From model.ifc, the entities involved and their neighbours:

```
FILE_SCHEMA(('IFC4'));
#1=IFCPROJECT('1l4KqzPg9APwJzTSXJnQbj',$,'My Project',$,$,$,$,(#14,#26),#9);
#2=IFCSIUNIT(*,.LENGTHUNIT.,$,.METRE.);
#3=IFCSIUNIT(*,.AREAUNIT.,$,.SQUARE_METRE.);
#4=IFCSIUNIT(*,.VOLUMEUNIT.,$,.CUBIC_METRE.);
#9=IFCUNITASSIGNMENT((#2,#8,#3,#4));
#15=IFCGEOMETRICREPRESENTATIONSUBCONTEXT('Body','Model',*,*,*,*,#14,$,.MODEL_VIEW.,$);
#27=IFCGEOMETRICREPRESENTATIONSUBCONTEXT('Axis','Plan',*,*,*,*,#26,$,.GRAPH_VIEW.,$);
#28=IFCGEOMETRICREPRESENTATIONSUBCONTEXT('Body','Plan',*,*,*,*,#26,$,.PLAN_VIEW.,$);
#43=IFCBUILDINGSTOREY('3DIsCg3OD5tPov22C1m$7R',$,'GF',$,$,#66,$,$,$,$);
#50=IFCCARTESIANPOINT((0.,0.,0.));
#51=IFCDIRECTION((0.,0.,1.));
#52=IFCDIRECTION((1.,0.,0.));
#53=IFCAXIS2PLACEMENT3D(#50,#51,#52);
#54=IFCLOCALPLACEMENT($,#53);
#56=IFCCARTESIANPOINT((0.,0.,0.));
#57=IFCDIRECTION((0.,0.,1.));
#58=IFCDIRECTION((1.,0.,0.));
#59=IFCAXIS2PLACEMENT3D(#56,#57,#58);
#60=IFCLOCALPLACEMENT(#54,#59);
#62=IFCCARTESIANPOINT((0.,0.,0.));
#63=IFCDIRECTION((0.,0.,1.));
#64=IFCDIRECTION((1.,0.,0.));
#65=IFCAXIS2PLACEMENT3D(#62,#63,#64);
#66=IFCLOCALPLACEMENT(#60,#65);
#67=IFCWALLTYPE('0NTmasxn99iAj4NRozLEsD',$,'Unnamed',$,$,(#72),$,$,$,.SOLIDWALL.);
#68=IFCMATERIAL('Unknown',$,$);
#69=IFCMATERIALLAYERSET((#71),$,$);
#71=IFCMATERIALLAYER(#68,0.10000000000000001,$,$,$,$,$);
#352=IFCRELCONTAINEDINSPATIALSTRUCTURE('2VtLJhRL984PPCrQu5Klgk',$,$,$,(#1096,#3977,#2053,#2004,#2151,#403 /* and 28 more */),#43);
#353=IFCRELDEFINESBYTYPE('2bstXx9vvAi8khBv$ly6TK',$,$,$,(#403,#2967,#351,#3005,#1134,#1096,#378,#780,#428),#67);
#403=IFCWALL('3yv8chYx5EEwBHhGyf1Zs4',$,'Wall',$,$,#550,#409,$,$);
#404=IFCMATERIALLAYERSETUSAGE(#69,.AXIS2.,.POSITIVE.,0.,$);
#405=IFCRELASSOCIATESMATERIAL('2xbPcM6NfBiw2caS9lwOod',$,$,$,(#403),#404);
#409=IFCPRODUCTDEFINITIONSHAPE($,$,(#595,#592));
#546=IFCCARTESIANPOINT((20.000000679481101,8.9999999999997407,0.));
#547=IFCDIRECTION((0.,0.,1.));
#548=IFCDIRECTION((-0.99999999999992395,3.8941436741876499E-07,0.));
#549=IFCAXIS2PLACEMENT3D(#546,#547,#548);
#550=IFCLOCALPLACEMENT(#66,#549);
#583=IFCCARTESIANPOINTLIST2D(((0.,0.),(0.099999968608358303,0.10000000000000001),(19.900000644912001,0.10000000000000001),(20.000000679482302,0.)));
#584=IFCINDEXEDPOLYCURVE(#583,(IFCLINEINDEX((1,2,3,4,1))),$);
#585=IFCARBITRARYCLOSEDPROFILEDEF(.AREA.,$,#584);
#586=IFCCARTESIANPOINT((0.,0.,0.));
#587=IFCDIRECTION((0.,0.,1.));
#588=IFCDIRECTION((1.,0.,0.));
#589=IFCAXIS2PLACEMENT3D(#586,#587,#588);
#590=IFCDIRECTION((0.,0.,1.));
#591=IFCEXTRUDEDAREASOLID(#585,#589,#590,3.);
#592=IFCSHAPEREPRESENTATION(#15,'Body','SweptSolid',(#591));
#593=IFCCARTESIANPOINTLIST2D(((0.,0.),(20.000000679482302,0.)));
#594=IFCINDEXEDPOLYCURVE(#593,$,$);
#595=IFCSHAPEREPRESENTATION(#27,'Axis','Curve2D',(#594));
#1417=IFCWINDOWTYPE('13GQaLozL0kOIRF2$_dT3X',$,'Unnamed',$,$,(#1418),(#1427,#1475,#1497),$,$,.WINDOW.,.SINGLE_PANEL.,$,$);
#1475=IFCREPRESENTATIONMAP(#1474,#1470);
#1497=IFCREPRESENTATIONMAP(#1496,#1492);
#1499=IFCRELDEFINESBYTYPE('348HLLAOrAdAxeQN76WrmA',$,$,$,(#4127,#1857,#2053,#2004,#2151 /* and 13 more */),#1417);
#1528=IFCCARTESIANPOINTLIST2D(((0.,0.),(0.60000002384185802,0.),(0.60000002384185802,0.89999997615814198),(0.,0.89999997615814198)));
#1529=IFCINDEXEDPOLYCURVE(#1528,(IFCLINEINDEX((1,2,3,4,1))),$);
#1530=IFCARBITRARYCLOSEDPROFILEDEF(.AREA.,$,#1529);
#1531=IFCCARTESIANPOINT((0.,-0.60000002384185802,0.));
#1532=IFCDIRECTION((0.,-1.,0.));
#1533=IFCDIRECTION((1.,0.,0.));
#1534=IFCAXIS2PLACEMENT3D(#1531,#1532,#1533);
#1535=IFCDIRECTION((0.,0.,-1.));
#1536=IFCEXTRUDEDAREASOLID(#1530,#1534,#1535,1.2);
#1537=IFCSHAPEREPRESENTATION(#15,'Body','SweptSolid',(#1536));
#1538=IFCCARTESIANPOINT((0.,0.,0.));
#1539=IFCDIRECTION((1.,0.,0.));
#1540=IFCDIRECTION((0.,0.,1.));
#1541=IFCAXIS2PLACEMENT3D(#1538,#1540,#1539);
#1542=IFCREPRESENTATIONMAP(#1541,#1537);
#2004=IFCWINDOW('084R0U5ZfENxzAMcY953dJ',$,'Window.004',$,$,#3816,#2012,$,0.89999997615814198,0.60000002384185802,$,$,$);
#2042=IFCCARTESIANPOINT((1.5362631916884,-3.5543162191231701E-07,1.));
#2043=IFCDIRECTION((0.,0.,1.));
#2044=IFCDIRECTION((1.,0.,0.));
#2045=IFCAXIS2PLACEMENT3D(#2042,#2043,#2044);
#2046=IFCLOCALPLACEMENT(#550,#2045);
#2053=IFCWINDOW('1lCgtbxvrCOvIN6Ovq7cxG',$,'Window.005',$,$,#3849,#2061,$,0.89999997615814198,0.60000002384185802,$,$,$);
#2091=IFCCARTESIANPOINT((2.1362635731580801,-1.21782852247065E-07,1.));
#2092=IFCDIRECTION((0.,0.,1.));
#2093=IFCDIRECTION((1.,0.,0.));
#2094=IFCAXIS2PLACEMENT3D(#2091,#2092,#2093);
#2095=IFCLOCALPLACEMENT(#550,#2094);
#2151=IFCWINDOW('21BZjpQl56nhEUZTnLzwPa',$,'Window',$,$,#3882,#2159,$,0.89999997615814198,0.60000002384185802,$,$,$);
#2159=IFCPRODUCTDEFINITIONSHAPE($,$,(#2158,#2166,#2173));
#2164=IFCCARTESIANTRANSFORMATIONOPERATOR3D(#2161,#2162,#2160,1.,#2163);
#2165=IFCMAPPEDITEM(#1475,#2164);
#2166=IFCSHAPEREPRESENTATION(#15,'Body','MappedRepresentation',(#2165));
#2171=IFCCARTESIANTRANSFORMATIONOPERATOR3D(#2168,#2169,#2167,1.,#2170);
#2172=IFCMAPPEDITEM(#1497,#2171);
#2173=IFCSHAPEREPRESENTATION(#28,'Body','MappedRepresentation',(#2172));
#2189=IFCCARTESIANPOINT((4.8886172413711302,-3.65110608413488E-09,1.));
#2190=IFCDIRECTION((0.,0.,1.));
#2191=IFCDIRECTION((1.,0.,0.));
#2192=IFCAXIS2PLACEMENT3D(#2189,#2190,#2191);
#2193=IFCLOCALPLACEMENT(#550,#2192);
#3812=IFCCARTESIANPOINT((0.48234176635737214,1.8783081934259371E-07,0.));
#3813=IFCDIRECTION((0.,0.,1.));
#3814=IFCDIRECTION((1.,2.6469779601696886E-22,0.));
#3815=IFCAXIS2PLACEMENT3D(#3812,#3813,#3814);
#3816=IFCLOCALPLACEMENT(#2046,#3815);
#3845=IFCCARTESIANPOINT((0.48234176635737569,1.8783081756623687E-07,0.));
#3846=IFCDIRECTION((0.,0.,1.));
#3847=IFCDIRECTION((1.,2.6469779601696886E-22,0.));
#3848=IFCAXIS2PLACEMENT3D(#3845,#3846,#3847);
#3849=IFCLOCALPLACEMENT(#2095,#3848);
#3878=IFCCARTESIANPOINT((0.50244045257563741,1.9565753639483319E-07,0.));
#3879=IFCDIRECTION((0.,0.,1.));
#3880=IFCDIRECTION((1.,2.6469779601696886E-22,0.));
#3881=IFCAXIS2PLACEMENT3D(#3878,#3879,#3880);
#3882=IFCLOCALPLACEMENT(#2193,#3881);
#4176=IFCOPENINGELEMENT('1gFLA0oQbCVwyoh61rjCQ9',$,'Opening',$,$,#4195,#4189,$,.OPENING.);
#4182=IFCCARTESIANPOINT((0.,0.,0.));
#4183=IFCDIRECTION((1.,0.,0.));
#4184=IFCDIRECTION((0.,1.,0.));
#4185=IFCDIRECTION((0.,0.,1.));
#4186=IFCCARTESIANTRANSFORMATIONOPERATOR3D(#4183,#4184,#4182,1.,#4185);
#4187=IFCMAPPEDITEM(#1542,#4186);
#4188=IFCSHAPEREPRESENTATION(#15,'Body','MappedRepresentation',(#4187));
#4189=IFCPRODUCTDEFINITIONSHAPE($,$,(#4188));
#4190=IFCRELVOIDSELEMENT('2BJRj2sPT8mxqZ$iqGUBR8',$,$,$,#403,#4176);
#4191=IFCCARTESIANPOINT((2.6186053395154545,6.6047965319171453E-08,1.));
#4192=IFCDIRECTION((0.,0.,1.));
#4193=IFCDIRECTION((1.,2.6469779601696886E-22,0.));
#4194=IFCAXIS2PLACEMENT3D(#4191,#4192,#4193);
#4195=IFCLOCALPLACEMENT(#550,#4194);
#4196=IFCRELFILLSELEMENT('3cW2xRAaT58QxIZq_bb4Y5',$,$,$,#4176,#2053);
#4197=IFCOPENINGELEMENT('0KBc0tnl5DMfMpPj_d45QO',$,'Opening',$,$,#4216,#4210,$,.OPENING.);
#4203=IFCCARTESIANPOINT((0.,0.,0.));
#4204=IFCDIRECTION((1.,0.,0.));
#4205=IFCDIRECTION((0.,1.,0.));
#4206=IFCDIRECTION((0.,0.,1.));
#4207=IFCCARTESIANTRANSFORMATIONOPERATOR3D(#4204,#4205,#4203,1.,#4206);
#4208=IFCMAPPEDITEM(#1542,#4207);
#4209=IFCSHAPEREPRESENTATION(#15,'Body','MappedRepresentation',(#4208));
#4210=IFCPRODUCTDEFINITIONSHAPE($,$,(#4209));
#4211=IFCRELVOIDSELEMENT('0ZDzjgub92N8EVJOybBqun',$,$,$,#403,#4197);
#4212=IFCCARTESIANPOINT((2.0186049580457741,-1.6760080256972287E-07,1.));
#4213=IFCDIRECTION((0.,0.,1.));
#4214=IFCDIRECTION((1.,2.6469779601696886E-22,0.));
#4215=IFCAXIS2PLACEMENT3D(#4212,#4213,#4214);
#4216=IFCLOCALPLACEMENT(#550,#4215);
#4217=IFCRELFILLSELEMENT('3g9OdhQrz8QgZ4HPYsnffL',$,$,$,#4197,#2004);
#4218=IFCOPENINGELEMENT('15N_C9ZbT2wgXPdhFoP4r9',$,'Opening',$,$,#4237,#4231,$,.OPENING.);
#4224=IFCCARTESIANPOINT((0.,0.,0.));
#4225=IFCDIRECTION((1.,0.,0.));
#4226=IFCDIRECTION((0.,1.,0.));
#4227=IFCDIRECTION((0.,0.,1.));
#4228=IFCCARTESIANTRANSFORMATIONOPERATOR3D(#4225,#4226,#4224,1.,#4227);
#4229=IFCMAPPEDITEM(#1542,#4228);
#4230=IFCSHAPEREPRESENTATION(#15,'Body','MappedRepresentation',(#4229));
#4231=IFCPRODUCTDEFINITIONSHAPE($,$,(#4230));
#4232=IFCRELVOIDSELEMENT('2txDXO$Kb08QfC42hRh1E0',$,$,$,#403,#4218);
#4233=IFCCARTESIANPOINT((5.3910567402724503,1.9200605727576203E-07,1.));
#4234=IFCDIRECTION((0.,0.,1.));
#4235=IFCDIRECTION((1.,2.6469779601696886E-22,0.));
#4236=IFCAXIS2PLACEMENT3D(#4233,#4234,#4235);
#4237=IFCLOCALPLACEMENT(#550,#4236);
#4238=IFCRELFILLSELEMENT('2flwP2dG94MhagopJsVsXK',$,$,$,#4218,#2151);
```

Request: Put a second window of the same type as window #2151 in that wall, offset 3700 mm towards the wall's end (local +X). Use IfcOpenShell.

```python
import ifcopenshell
import ifcopenshell.api.feature
import ifcopenshell.api.geometry
import ifcopenshell.api.root
import ifcopenshell.geom
import ifcopenshell.util.element
import ifcopenshell.util.placement
import ifcopenshell.util.shape
import ifcopenshell.util.unit

model = ifcopenshell.open("model.ifc")
unit_scale = ifcopenshell.util.unit.calculate_unit_scale(model)
settings = ifcopenshell.geom.settings()


def volume(element):
    """Net volume in cubic metres, openings subtracted."""
    shape = ifcopenshell.geom.create_shape(settings, element)
    return ifcopenshell.util.shape.get_volume(shape.geometry)


window = model.by_guid("21BZjpQl56nhEUZTnLzwPa")
opening = window.FillsVoids[0].RelatingOpeningElement
wall = opening.VoidsElements[0].RelatingBuildingElement
before = volume(wall)
shift = ifcopenshell.util.placement.get_local_placement(wall.ObjectPlacement)[:3, 0] * 3.7 / unit_scale

# copy_class copies the void relationship, type, container and properties, but no geometry.
new_opening = ifcopenshell.api.root.copy_class(model, product=opening)
new_opening.Representation = ifcopenshell.util.element.copy_deep(
    model, opening.Representation, exclude=["IfcGeometricRepresentationContext", "IfcRepresentationMap"]
)
new_window = ifcopenshell.api.root.copy_class(model, product=window)
new_window.Representation = ifcopenshell.util.element.copy_deep(
    model, window.Representation, exclude=["IfcGeometricRepresentationContext", "IfcRepresentationMap"]
)
ifcopenshell.api.feature.add_filling(model, opening=new_opening, element=new_window)

for old, new in ((opening, new_opening), (window, new_window)):
    matrix = ifcopenshell.util.placement.get_local_placement(old.ObjectPlacement)
    matrix[:3, 3] += shift
    ifcopenshell.api.geometry.edit_object_placement(model, product=new, matrix=matrix, is_si=False)

after = volume(wall)

print(f"wall volume {before:.3f} -> {after:.3f} m3")

model.write("model-out.ifc")
```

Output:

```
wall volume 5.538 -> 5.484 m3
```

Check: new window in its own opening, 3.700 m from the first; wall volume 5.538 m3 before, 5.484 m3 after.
